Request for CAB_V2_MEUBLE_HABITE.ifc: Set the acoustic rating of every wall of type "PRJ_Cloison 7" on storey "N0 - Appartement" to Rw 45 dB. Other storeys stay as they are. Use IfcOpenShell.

First a look at what the model holds.

```python
import ifcopenshell
import ifcopenshell.util.element

model = ifcopenshell.open("CAB_V2_MEUBLE_HABITE.ifc")
print(model.schema)
storey = next(s for s in model.by_type("IfcBuildingStorey") if s.Name == "N0 - Appartement")
walls = [e for e in ifcopenshell.util.element.get_decomposition(storey) if e.is_a("IfcWall")]
seen = {}
for e in walls:
    element_type = ifcopenshell.util.element.get_type(e)
    key = (element_type.Name if element_type != e and element_type else None, ifcopenshell.util.element.get_pset(e, "Pset_WallCommon", "AcousticRating"))
    seen[key] = seen.get(key, 0) + 1
for (name, value), count in sorted(seen.items(), key=str):
    print(count, "x", name, "|", value)
```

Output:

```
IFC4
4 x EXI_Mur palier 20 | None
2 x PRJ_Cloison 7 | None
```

```python
import ifcopenshell
import ifcopenshell.api.pset
import ifcopenshell.util.element

model = ifcopenshell.open("CAB_V2_MEUBLE_HABITE.ifc")

storey = next(s for s in model.by_type("IfcBuildingStorey") if s.Name == "N0 - Appartement")
walls = [e for e in ifcopenshell.util.element.get_decomposition(storey) if e.is_a("IfcWall")]

count = 0
for e in walls:
    element_type = ifcopenshell.util.element.get_type(e)
    if element_type in (None, e) or element_type.Name != "PRJ_Cloison 7":
        continue
    # add_pset returns the element's existing set when there is one.
    pset = ifcopenshell.api.pset.add_pset(model, product=e, name="Pset_WallCommon")
    ifcopenshell.api.pset.edit_pset(model, pset=pset, properties={"AcousticRating": "Rw 45 dB"})
    count += 1

print(count, "walls updated")

model.write("CAB_V2_MEUBLE_HABITE_rev.ifc")
```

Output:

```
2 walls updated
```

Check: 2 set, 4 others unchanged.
